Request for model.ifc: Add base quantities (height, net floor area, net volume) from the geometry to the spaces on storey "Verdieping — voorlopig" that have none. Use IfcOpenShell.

First a look at what the model holds.

```python
import ifcopenshell
import ifcopenshell.util.element
import ifcopenshell.util.unit

model = ifcopenshell.open("model.ifc")
print(model.schema)
for unit_type in ("LENGTHUNIT", "AREAUNIT", "VOLUMEUNIT"):
    print(unit_type, ifcopenshell.util.unit.calculate_unit_scale(model, unit_type))
storey = next(s for s in model.by_type("IfcBuildingStorey") if s.Name == "Verdieping — voorlopig")
spaces = [e for e in ifcopenshell.util.element.get_decomposition(storey) if e.is_a("IfcSpace")]
for e in sorted(spaces, key=lambda e: e.id()):
    print(e.id(), e.is_a(), e.Name, list(ifcopenshell.util.element.get_psets(e, qtos_only=True)), sep=" | ")
```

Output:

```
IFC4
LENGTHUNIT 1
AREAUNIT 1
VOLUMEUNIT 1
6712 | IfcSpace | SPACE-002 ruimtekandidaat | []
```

```python
import ifcopenshell
import ifcopenshell.api.pset
import ifcopenshell.geom
import ifcopenshell.util.element
import ifcopenshell.util.shape
import ifcopenshell.util.unit

model = ifcopenshell.open("model.ifc")
unit_scale = ifcopenshell.util.unit.calculate_unit_scale(model)
area_scale = ifcopenshell.util.unit.calculate_unit_scale(model, "AREAUNIT")
volume_scale = ifcopenshell.util.unit.calculate_unit_scale(model, "VOLUMEUNIT")
settings = ifcopenshell.geom.settings()

storey = next(s for s in model.by_type("IfcBuildingStorey") if s.Name == "Verdieping — voorlopig")
spaces = [e for e in ifcopenshell.util.element.get_decomposition(storey) if e.is_a("IfcSpace")]

for e in sorted(spaces, key=lambda e: e.id()):
    if ifcopenshell.util.element.get_psets(e, qtos_only=True, should_inherit=False):
        continue
    # Geometry comes back in metres, in the element's own axes.
    shape = ifcopenshell.geom.create_shape(settings, e)
    values = {
        "Height": ifcopenshell.util.shape.get_z(shape.geometry) / unit_scale,
        "NetFloorArea": ifcopenshell.util.shape.get_footprint_area(shape.geometry) / area_scale,
        "NetVolume": ifcopenshell.util.shape.get_volume(shape.geometry) / volume_scale,
    }
    qto = ifcopenshell.api.pset.add_qto(model, product=e, name="Qto_SpaceBaseQuantities")
    ifcopenshell.api.pset.edit_qto(model, qto=qto, properties=values)
    print(e.id(), {k: round(v, 3) for k, v in values.items()})

model.write("model_edited.ifc")
```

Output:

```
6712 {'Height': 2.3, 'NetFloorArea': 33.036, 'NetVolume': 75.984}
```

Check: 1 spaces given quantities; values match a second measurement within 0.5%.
